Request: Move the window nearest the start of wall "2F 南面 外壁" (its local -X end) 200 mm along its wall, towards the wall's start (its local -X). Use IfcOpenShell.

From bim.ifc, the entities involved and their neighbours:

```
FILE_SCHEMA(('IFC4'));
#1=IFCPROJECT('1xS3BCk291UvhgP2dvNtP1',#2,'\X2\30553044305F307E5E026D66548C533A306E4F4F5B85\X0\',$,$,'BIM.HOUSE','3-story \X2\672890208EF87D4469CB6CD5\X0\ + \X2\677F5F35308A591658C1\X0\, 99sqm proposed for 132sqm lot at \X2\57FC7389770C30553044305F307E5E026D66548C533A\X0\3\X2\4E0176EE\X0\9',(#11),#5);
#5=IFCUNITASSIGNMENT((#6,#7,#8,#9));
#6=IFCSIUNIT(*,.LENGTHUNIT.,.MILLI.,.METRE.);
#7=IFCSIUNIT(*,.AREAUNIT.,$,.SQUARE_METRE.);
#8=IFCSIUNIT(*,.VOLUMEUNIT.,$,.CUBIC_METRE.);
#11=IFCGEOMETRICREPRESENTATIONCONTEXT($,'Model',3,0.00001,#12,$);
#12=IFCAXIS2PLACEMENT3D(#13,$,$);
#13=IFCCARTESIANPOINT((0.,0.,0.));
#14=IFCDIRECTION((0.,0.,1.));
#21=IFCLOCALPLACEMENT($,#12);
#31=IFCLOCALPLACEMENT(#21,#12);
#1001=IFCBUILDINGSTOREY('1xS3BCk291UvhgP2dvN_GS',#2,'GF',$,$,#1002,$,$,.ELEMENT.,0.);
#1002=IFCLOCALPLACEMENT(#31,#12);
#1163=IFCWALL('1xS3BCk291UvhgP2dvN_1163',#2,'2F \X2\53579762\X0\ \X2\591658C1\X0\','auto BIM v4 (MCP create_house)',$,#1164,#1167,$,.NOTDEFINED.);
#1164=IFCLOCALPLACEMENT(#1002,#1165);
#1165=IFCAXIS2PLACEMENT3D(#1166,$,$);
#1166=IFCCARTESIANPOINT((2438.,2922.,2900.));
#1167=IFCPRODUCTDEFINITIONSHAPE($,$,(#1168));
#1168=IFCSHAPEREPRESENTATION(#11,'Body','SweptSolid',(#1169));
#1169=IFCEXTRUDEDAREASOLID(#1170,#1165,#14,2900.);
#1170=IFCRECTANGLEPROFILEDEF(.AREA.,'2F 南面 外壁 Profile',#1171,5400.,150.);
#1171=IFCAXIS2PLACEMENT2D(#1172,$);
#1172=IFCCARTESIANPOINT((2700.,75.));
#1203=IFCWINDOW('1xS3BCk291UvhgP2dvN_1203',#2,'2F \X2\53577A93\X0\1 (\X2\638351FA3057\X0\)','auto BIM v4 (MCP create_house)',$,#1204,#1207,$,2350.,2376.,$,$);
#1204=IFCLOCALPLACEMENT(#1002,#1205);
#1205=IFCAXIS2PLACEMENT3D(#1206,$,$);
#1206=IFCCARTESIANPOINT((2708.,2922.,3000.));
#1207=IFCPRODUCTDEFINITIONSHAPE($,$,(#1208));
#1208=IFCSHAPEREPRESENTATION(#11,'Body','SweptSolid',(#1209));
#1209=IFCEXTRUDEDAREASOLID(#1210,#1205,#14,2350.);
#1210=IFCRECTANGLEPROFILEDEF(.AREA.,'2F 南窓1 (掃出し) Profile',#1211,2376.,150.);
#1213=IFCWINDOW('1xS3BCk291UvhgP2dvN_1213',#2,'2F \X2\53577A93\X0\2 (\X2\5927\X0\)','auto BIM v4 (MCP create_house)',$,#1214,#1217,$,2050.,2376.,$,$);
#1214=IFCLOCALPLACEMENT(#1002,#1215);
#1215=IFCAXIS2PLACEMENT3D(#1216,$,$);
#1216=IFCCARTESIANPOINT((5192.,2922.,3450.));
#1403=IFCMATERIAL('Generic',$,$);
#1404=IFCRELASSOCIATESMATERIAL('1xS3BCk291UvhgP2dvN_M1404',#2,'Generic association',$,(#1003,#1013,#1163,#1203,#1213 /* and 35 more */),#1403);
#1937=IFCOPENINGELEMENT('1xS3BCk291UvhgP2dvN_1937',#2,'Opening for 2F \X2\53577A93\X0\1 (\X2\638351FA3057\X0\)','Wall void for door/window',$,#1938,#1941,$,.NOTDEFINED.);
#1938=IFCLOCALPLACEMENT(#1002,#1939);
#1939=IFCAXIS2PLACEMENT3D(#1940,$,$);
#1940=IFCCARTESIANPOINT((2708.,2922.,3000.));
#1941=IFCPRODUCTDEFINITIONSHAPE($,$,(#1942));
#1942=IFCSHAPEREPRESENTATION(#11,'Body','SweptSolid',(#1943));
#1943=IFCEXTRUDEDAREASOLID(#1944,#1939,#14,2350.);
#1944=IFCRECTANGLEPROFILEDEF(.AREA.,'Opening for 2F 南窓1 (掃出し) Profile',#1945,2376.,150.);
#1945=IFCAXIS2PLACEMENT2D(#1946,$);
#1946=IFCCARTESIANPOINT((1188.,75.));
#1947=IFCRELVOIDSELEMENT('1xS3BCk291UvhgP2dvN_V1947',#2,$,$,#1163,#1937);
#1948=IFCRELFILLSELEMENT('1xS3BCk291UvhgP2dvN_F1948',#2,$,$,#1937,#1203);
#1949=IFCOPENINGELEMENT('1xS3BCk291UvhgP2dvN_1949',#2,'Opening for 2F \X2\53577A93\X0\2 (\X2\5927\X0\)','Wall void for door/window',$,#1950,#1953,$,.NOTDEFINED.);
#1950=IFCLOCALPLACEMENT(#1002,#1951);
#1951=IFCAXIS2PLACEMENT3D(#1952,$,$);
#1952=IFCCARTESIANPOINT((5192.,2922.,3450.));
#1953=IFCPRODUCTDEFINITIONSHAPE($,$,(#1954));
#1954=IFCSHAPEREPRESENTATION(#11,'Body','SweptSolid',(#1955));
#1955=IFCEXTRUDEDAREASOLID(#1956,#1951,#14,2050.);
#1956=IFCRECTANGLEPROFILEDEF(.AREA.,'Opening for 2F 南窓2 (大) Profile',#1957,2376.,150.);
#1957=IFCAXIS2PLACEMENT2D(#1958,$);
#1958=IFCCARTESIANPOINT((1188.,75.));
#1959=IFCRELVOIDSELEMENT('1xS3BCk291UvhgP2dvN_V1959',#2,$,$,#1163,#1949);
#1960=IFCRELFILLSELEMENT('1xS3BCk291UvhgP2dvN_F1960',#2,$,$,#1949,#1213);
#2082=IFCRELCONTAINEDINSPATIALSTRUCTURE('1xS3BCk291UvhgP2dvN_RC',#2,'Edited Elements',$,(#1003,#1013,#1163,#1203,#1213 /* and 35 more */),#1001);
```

```python
import ifcopenshell
import ifcopenshell.api.geometry
import ifcopenshell.util.placement

model = ifcopenshell.open("bim.ifc")

window = model.by_guid("1xS3BCk291UvhgP2dvN_1203")
opening = window.FillsVoids[0].RelatingOpeningElement
wall = opening.VoidsElements[0].RelatingBuildingElement

wall_matrix = ifcopenshell.util.placement.get_local_placement(wall.ObjectPlacement)
shift = wall_matrix[:3, 0] * -200.0
before = ifcopenshell.util.placement.get_local_placement(window.ObjectPlacement)[:3, 3].copy()

# The window is not placed relative to its opening, so move both.
for product in (opening, window):
    matrix = ifcopenshell.util.placement.get_local_placement(product.ObjectPlacement)
    matrix[:3, 3] += shift
    ifcopenshell.api.geometry.edit_object_placement(model, product=product, matrix=matrix, is_si=False)

after = ifcopenshell.util.placement.get_local_placement(window.ObjectPlacement)[:3, 3]
print("window moved by", (after - before).round(3) + 0.0)

model.write("bim-out.ifc")
```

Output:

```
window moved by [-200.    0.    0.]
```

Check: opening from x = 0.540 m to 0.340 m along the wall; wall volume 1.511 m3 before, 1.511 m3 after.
